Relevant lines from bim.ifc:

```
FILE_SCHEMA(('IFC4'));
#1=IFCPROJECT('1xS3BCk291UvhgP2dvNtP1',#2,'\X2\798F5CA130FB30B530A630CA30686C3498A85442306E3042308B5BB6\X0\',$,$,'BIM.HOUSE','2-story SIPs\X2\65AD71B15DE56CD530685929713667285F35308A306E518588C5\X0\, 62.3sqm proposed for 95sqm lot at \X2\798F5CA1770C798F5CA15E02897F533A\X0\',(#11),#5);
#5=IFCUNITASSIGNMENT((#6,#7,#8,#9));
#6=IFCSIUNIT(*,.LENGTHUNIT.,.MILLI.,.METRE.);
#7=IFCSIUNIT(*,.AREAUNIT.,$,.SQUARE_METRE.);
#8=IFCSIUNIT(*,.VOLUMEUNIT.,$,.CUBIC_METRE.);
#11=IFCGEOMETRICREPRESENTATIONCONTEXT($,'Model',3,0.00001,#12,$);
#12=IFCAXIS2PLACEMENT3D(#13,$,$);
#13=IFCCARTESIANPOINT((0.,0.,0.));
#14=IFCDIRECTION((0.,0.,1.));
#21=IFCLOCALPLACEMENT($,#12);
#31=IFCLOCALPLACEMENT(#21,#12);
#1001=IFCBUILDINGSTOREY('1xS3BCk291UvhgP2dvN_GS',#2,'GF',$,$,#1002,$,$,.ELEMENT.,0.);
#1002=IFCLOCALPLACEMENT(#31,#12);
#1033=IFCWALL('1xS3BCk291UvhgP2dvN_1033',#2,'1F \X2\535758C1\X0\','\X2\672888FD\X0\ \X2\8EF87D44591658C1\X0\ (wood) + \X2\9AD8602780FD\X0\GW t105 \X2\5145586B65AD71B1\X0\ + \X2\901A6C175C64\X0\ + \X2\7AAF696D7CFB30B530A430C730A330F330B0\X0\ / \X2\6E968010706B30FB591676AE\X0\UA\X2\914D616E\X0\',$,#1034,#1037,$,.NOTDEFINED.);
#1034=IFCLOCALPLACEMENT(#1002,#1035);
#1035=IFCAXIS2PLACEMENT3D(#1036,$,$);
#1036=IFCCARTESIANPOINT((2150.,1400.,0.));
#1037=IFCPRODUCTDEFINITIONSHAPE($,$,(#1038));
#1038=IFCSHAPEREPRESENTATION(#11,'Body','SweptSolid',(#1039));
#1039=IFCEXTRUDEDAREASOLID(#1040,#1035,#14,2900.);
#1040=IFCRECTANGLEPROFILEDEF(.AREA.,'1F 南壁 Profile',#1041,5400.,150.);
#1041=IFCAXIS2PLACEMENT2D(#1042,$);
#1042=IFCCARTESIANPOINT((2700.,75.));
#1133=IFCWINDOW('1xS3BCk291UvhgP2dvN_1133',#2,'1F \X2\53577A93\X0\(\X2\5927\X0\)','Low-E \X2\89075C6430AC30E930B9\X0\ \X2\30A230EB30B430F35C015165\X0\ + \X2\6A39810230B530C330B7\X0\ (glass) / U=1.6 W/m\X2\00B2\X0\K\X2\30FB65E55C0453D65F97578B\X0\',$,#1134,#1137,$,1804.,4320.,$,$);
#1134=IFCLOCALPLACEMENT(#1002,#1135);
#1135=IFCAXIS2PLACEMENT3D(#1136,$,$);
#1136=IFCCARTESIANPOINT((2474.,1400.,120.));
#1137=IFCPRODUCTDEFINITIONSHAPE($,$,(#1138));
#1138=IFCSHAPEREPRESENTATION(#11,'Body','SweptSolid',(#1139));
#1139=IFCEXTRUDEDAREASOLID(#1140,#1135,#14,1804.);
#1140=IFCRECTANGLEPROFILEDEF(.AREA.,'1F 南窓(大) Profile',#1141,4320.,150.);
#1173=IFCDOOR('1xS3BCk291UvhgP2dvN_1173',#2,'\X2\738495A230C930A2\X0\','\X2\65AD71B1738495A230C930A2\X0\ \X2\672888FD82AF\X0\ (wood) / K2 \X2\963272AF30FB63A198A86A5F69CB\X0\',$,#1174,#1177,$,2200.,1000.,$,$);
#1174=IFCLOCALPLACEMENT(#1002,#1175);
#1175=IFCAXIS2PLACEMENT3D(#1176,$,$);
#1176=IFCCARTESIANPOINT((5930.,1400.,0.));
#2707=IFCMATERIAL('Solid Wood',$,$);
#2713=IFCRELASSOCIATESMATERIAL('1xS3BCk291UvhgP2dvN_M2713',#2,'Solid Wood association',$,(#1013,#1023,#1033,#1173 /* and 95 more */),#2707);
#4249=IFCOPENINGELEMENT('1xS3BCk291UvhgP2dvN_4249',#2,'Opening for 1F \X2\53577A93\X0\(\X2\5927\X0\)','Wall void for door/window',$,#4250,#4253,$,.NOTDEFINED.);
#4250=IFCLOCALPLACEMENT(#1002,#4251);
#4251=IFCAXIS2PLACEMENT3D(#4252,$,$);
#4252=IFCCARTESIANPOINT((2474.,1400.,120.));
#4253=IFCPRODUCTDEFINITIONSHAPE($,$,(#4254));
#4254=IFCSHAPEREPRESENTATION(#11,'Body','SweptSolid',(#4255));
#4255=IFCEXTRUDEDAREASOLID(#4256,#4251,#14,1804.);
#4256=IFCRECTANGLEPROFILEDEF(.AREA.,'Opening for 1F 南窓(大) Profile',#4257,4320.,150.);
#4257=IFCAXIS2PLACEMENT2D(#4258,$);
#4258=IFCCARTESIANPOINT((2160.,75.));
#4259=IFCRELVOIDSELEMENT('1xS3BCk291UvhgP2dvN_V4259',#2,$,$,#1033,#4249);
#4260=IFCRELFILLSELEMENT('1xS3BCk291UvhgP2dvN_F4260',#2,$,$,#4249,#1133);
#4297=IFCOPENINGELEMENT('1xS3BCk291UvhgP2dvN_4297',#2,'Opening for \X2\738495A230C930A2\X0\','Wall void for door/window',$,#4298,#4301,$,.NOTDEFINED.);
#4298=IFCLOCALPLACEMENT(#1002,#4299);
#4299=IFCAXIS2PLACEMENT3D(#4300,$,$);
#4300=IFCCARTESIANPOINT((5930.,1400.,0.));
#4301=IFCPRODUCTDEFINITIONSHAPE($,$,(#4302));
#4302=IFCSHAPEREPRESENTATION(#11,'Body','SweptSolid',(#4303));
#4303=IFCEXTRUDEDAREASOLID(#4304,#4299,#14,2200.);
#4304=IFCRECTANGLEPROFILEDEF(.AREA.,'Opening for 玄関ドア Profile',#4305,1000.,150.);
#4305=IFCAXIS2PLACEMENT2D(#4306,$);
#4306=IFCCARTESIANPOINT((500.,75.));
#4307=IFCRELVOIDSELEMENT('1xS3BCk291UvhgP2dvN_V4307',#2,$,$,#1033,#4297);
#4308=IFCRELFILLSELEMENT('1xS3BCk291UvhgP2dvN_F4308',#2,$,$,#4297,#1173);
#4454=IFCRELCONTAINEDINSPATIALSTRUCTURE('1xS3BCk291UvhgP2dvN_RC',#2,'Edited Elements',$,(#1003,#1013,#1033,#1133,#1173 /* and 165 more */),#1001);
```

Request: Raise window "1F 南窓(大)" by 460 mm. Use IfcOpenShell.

```python
import numpy as np
import ifcopenshell
import ifcopenshell.api.geometry
import ifcopenshell.util.placement
import ifcopenshell.util.unit

model = ifcopenshell.open("bim.ifc")
unit_scale = ifcopenshell.util.unit.calculate_unit_scale(model)

window = model.by_guid("1xS3BCk291UvhgP2dvN_1133")
opening = window.FillsVoids[0].RelatingOpeningElement
dz = 460.0

shift = np.array([0.0, 0.0, dz])
# The window is not placed relative to its opening, so move both.
for product in (opening, window):
    matrix = ifcopenshell.util.placement.get_local_placement(product.ObjectPlacement)
    matrix[:3, 3] += shift
    ifcopenshell.api.geometry.edit_object_placement(model, product=product, matrix=matrix, is_si=False)

print(f"moved by {dz * unit_scale:+.3f} m")

model.write("bim_updated.ifc")
```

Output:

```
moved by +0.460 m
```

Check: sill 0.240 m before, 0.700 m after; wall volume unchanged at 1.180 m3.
